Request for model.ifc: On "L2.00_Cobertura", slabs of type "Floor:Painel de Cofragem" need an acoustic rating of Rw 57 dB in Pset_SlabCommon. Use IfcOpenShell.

First a look at what the model holds.

```python
import ifcopenshell
import ifcopenshell.util.element

model = ifcopenshell.open("model.ifc")
print(model.schema)
storey = next(s for s in model.by_type("IfcBuildingStorey") if s.Name == "L2.00_Cobertura")
slabs = [e for e in ifcopenshell.util.element.get_decomposition(storey) if e.is_a("IfcSlab")]
seen = {}
for e in slabs:
    element_type = ifcopenshell.util.element.get_type(e)
    key = (element_type.Name if element_type != e and element_type else None, ifcopenshell.util.element.get_pset(e, "Pset_SlabCommon", "AcousticRating"))
    seen[key] = seen.get(key, 0) + 1
for (name, value), count in sorted(seen.items(), key=str):
    print(count, "x", name, "|", value)
```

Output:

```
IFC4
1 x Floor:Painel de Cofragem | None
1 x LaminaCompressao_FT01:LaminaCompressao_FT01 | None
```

```python
import ifcopenshell
import ifcopenshell.api.pset
import ifcopenshell.util.element

model = ifcopenshell.open("model.ifc")

storey = next(s for s in model.by_type("IfcBuildingStorey") if s.Name == "L2.00_Cobertura")
slabs = [e for e in ifcopenshell.util.element.get_decomposition(storey) if e.is_a("IfcSlab")]

count = 0
for e in slabs:
    element_type = ifcopenshell.util.element.get_type(e)
    if element_type in (None, e) or element_type.Name != "Floor:Painel de Cofragem":
        continue
    # add_pset returns the element's existing set when there is one.
    pset = ifcopenshell.api.pset.add_pset(model, product=e, name="Pset_SlabCommon")
    ifcopenshell.api.pset.edit_pset(model, pset=pset, properties={"AcousticRating": "Rw 57 dB"})
    count += 1

print(count, "slabs updated")

model.write("model_v2.ifc")
```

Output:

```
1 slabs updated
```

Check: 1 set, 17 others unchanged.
